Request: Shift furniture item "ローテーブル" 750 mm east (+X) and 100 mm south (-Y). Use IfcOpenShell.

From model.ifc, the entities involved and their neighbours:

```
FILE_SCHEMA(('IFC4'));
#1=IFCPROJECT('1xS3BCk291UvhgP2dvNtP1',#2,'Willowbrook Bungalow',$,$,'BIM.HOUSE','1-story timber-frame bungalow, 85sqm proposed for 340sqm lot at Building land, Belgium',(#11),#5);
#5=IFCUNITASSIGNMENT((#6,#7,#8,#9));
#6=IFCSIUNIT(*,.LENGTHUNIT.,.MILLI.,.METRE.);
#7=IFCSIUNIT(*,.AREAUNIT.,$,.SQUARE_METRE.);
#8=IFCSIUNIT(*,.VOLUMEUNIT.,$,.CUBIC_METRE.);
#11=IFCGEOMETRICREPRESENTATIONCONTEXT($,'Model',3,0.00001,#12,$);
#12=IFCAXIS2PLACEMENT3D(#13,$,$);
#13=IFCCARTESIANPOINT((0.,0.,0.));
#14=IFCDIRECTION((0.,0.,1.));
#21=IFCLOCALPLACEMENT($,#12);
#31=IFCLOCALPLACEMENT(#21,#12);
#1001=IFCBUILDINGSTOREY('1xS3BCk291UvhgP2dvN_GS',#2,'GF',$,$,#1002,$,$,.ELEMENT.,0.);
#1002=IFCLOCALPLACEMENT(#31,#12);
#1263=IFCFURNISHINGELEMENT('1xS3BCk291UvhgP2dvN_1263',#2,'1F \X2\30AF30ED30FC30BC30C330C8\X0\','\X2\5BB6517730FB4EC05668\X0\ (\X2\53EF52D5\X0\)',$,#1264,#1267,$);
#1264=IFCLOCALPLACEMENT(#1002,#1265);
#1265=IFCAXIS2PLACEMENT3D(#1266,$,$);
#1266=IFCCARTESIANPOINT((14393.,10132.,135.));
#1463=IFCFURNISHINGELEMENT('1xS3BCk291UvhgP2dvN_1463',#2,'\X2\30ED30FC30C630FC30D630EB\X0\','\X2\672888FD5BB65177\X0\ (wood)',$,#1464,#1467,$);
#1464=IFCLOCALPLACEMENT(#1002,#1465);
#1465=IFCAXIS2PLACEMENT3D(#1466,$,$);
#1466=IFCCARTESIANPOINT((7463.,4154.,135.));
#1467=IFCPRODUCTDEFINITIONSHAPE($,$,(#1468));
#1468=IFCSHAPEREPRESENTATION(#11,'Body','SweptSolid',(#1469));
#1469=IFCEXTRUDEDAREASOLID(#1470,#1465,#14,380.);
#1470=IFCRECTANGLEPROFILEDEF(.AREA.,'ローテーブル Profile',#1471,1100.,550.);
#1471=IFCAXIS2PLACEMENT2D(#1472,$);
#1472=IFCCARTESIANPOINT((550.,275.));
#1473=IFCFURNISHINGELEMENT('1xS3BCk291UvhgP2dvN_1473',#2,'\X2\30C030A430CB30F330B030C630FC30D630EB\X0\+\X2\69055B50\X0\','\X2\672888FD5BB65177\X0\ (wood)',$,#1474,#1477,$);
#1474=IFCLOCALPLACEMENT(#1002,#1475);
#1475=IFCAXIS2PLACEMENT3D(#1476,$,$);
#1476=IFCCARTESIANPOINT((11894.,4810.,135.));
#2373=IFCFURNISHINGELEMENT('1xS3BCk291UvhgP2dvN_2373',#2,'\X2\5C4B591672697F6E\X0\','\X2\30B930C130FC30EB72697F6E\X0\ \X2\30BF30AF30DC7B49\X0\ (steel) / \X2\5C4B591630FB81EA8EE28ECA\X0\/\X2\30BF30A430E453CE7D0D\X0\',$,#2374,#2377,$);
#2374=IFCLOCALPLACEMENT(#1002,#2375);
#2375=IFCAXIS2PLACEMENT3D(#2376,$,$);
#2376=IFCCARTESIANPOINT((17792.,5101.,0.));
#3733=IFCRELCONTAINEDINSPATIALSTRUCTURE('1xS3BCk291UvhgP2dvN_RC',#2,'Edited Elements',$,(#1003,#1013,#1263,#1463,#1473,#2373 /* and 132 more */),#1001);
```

```python
import ifcopenshell
import ifcopenshell.api.geometry
import ifcopenshell.util.placement

model = ifcopenshell.open("model.ifc")

item = model.by_guid("1xS3BCk291UvhgP2dvN_1463")
matrix = ifcopenshell.util.placement.get_local_placement(item.ObjectPlacement)
matrix[0, 3] += 750.0
matrix[1, 3] -= 100.0
ifcopenshell.api.geometry.edit_object_placement(model, product=item, matrix=matrix, is_si=False)

print(ifcopenshell.util.placement.get_local_placement(item.ObjectPlacement).round(3) + 0.0)

model.write("model-out.ifc")
```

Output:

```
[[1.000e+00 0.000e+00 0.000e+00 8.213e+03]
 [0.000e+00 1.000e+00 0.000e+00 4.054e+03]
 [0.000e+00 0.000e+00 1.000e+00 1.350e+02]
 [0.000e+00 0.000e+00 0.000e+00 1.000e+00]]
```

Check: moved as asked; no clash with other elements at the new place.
